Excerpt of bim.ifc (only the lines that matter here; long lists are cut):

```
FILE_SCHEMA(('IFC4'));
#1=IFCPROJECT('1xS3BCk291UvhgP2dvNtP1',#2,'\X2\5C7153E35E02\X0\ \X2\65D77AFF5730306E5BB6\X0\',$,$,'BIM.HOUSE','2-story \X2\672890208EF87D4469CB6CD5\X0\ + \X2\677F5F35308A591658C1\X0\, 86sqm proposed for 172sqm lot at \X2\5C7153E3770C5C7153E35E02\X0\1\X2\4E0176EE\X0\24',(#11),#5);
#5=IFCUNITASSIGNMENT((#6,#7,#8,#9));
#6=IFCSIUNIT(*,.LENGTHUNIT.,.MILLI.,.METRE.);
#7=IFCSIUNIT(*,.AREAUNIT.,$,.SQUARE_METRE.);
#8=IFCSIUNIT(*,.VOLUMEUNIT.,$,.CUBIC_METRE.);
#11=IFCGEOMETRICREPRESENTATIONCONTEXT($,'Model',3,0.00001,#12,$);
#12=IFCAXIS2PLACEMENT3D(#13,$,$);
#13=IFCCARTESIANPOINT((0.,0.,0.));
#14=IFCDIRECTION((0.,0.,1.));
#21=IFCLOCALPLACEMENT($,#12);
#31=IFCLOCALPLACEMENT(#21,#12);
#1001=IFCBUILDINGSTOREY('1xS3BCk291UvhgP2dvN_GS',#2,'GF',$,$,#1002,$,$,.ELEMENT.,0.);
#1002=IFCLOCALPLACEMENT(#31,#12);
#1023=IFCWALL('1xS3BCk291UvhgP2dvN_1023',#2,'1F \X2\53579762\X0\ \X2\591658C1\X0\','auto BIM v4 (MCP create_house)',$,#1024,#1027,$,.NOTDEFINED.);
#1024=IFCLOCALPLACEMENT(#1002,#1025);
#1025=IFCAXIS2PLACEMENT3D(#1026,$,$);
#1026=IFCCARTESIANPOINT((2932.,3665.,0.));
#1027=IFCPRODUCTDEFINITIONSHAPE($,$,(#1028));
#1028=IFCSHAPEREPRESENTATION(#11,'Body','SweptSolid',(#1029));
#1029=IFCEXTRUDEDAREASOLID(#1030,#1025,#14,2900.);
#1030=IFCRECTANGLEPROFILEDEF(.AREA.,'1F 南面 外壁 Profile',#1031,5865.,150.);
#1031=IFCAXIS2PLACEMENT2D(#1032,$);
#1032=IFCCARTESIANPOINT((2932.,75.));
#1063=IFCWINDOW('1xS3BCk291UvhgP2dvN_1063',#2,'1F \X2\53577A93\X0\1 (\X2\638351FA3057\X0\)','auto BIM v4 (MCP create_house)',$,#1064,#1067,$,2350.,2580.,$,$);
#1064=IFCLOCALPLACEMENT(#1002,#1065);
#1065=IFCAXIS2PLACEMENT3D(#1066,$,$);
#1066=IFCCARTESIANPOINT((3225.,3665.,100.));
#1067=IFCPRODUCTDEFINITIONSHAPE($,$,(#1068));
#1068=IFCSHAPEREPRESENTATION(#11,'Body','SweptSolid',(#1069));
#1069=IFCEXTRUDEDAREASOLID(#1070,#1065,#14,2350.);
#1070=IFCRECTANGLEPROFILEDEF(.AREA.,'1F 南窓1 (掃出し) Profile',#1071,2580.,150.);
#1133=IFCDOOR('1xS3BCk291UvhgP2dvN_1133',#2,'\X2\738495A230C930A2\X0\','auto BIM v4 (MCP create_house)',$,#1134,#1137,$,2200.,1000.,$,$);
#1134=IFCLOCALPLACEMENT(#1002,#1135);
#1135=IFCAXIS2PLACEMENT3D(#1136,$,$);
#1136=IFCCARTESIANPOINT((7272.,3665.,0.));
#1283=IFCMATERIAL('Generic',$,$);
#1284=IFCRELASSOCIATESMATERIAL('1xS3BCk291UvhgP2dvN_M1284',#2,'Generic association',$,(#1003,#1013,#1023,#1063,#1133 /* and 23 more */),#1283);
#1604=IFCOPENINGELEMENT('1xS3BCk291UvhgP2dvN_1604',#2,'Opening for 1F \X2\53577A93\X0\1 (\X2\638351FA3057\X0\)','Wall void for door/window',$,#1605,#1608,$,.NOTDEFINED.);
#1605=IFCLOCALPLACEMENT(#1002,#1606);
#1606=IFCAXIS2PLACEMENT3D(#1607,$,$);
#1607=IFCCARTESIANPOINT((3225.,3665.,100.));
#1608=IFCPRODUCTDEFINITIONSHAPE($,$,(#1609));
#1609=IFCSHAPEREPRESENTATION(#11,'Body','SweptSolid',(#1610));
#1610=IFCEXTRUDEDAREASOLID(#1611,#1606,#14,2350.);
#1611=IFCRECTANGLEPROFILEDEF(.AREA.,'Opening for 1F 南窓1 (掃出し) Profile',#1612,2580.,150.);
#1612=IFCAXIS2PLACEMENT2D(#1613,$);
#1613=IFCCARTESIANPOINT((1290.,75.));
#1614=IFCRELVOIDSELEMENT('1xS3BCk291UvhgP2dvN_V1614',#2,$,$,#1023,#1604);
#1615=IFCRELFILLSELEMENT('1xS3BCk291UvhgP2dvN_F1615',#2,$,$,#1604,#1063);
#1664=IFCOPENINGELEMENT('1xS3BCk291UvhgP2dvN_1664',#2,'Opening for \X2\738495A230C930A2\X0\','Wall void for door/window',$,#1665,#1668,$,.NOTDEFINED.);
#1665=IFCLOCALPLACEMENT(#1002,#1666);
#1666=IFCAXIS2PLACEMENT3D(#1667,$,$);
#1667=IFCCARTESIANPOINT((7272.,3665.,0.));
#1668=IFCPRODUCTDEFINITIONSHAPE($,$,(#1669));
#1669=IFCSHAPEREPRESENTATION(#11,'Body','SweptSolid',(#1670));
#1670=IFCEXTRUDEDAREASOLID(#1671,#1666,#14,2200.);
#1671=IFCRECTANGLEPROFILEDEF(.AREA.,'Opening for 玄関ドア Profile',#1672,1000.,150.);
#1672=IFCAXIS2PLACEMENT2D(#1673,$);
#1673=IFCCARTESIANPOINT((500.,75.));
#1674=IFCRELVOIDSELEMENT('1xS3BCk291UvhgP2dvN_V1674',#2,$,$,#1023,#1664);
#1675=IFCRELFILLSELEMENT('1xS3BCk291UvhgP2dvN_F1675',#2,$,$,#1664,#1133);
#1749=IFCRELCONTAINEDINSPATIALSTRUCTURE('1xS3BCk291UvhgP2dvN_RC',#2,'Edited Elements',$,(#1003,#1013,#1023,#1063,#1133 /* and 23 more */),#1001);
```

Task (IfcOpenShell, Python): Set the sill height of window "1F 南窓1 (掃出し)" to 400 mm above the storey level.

```python
import numpy as np
import ifcopenshell
import ifcopenshell.api.geometry
import ifcopenshell.geom
import ifcopenshell.util.element
import ifcopenshell.util.placement
import ifcopenshell.util.shape
import ifcopenshell.util.unit

model = ifcopenshell.open("bim.ifc")
unit_scale = ifcopenshell.util.unit.calculate_unit_scale(model)

window = model.by_id(1063)
opening = window.FillsVoids[0].RelatingOpeningElement
storey = ifcopenshell.util.element.get_container(window, ifc_class="IfcBuildingStorey")
level = ifcopenshell.util.placement.get_local_placement(storey.ObjectPlacement)[2, 3]

# The opening's origin need not be at the sill, so measure its lowest point.
shape = ifcopenshell.geom.create_shape(ifcopenshell.geom.settings(), opening)
bottom = ifcopenshell.util.shape.get_shape_bottom_elevation(shape, shape.geometry) / unit_scale
dz = level + 400.0 - bottom

shift = np.array([0.0, 0.0, dz])
# The window is not placed relative to its opening, so move both.
for product in (opening, window):
    matrix = ifcopenshell.util.placement.get_local_placement(product.ObjectPlacement)
    matrix[:3, 3] += shift
    ifcopenshell.api.geometry.edit_object_placement(model, product=product, matrix=matrix, is_si=False)

print(f"moved by {dz * unit_scale:+.3f} m")

model.write("bim_rev.ifc")
```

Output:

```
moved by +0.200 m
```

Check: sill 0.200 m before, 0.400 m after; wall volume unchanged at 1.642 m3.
